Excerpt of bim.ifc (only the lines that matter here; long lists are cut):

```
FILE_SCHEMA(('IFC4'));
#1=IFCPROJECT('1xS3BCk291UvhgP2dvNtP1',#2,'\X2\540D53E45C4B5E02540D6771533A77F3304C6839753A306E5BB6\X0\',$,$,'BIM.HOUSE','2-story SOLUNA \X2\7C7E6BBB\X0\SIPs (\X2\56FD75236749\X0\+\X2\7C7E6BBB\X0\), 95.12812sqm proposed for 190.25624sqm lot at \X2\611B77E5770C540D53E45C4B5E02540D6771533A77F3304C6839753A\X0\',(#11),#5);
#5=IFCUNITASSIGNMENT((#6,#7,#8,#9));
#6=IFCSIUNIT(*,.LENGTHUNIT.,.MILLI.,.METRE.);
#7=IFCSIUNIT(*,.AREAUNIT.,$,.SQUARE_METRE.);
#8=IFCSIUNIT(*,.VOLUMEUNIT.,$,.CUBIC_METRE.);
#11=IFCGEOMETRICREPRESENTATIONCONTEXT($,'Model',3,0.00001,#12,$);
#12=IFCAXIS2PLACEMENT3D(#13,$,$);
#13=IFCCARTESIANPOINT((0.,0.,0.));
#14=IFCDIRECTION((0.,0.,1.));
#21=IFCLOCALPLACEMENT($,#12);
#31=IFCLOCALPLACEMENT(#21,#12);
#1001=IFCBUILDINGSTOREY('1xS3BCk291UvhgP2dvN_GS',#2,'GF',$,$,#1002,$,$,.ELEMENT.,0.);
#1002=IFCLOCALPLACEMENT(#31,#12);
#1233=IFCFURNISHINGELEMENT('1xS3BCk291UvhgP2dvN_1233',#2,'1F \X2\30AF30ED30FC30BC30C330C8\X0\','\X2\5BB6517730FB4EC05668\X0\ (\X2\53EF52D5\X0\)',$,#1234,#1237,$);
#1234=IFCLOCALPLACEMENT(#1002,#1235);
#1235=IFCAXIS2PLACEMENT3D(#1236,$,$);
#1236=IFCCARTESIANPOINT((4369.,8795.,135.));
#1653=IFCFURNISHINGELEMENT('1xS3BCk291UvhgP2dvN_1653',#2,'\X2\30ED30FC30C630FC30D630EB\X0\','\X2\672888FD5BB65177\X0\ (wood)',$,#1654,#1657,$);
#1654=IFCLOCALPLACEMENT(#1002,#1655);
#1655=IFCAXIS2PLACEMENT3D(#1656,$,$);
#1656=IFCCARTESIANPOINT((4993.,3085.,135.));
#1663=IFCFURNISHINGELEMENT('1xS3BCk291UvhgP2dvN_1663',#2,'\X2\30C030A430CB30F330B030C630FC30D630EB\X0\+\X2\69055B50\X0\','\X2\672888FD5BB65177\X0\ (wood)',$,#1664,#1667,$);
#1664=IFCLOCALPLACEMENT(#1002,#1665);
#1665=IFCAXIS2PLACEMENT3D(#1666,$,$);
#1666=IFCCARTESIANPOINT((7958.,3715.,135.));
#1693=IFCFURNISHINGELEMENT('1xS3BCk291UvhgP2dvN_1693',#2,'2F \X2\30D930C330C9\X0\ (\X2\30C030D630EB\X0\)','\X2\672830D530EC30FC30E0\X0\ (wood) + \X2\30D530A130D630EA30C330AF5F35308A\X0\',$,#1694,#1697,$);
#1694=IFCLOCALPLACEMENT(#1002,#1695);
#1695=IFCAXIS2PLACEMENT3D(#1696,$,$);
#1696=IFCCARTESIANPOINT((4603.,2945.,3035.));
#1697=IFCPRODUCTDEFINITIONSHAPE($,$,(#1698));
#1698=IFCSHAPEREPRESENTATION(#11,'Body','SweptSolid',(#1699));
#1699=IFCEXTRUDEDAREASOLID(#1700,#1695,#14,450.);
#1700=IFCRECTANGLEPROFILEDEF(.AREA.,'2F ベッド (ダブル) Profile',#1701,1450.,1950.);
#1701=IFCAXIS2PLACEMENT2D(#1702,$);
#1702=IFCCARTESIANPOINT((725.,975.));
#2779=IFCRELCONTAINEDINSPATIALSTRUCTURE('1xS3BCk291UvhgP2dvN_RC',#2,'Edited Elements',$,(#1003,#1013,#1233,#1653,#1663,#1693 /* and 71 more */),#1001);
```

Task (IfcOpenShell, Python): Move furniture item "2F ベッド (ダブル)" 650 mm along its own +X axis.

```python
import ifcopenshell
import ifcopenshell.api.geometry
import ifcopenshell.util.placement

model = ifcopenshell.open("bim.ifc")

item = model.by_guid("1xS3BCk291UvhgP2dvN_1693")
matrix = ifcopenshell.util.placement.get_local_placement(item.ObjectPlacement)
matrix[:3, 3] += matrix[:3, 0] * 650.0
ifcopenshell.api.geometry.edit_object_placement(model, product=item, matrix=matrix, is_si=False)

print(ifcopenshell.util.placement.get_local_placement(item.ObjectPlacement).round(3) + 0.0)

model.write("bim_rev.ifc")
```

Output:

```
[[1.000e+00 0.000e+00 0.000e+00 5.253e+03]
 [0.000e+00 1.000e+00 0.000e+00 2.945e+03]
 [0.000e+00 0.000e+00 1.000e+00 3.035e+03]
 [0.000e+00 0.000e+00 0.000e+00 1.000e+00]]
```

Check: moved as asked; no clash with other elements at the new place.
